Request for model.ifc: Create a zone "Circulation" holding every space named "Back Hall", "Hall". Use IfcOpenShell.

First a look at what the model holds.

```python
import ifcopenshell

model = ifcopenshell.open("model.ifc")
print(model.schema)
seen = {}
for space in model.by_type("IfcSpace"):
    seen[space.LongName] = seen.get(space.LongName, 0) + 1
for name, count in sorted(seen.items(), key=str):
    print(count, "x", name)
print("zones:", [z.Name for z in model.by_type("IfcZone")][:20])
```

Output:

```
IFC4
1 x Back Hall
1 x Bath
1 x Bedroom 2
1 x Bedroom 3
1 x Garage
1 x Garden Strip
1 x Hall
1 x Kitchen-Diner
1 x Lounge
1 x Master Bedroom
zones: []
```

```python
import ifcopenshell
import ifcopenshell.api.group
import ifcopenshell.api.root

model = ifcopenshell.open("model.ifc")

names = {"Back Hall", "Hall"}
spaces = [s for s in model.by_type("IfcSpace") if s.LongName in names]

zone = ifcopenshell.api.root.create_entity(model, ifc_class="IfcZone", name="Circulation")
ifcopenshell.api.group.assign_group(model, products=spaces, group=zone)
print(len(spaces), "spaces in", zone.Name)

model.write("model_v2.ifc")
```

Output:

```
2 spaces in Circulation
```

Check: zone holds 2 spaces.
